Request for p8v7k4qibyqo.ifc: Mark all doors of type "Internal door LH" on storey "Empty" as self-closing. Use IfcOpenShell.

First a look at what the model holds.

```python
import ifcopenshell
import ifcopenshell.util.element

model = ifcopenshell.open("p8v7k4qibyqo.ifc")
print(model.schema)
storey = next(s for s in model.by_type("IfcBuildingStorey") if s.Name == "Empty")
doors = [e for e in ifcopenshell.util.element.get_decomposition(storey) if e.is_a("IfcDoor")]
seen = {}
for e in doors:
    element_type = ifcopenshell.util.element.get_type(e)
    key = (element_type.Name if element_type != e and element_type else None, ifcopenshell.util.element.get_pset(e, "Pset_DoorCommon", "SelfClosing"))
    seen[key] = seen.get(key, 0) + 1
for (name, value), count in sorted(seen.items(), key=str):
    print(count, "x", name, "|", value)
```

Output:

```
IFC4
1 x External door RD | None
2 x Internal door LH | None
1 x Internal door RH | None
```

```python
import ifcopenshell
import ifcopenshell.api.pset
import ifcopenshell.util.element

model = ifcopenshell.open("p8v7k4qibyqo.ifc")

storey = next(s for s in model.by_type("IfcBuildingStorey") if s.Name == "Empty")
doors = [e for e in ifcopenshell.util.element.get_decomposition(storey) if e.is_a("IfcDoor")]

count = 0
for e in doors:
    element_type = ifcopenshell.util.element.get_type(e)
    if element_type in (None, e) or element_type.Name != "Internal door LH":
        continue
    # add_pset returns the element's existing set when there is one.
    pset = ifcopenshell.api.pset.add_pset(model, product=e, name="Pset_DoorCommon")
    ifcopenshell.api.pset.edit_pset(model, pset=pset, properties={"SelfClosing": True})
    count += 1

print(count, "doors updated")

model.write("p8v7k4qibyqo_rev.ifc")
```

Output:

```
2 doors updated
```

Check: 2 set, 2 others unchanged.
